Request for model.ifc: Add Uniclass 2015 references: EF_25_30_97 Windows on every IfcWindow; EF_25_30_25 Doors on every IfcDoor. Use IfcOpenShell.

First a look at what the model holds.

```python
import ifcopenshell

model = ifcopenshell.open("model.ifc")
print(model.schema)
print("classifications:", [c.Name for c in model.by_type("IfcClassification")])
for ifc_class in ("IfcDoor", "IfcRoof", "IfcStair", "IfcWall", "IfcWindow"):
    print(ifc_class, len(model.by_type(ifc_class)))
```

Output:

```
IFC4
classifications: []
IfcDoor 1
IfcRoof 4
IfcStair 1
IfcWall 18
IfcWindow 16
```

```python
import ifcopenshell
import ifcopenshell.api.classification

model = ifcopenshell.open("model.ifc")

system = ifcopenshell.api.classification.add_classification(model, classification="Uniclass 2015")

codes = {
    "IfcWindow": ("EF_25_30_97", "Windows"),
    "IfcDoor": ("EF_25_30_25", "Doors"),
}
for ifc_class, (code, name) in codes.items():
    products = model.by_type(ifc_class)
    ifcopenshell.api.classification.add_reference(
        model, products=products, classification=system, identification=code, name=name
    )
    print(code, len(products))

model.write("model-out.ifc")
```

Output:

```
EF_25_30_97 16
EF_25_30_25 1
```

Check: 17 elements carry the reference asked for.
